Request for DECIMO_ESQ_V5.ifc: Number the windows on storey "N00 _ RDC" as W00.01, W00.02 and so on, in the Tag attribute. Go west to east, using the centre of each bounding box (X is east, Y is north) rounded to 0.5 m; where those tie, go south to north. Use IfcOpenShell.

First a look at what the model holds.

```python
import ifcopenshell
import ifcopenshell.util.element
import ifcopenshell.util.placement

model = ifcopenshell.open("DECIMO_ESQ_V5.ifc")
print(model.schema)
storey = next(s for s in model.by_type("IfcBuildingStorey") if s.Name == "N00 _ RDC")
windows = [e for e in ifcopenshell.util.element.get_decomposition(storey) if e.is_a("IfcWindow")]
for e in sorted(windows, key=lambda e: e.id()):
    origin = ifcopenshell.util.placement.get_local_placement(e.ObjectPlacement)[:3, 3]
    print(e.id(), e.Tag, e.Name, origin.round(2) + 0.0, sep=" | ")
```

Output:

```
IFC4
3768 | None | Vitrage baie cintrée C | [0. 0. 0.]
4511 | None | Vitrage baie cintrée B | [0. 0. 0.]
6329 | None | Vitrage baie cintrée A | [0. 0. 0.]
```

```python
import ifcopenshell
import ifcopenshell.geom
import ifcopenshell.util.element
import ifcopenshell.util.shape

model = ifcopenshell.open("DECIMO_ESQ_V5.ifc")
settings = ifcopenshell.geom.settings()
settings.set("use-world-coords", True)


def centre(element):
    shape = ifcopenshell.geom.create_shape(settings, element)
    return ifcopenshell.util.shape.get_bbox_centroid(shape.geometry)


storey = next(s for s in model.by_type("IfcBuildingStorey") if s.Name == "N00 _ RDC")
windows = [e for e in ifcopenshell.util.element.get_decomposition(storey) if e.is_a("IfcWindow")]

# Insertion points can sit at a corner or the storey origin, so sort by the geometry (in metres).
centres = {e: centre(e) for e in windows}
windows.sort(key=lambda e: (round(centres[e][0] / 0.5), centres[e][1]))

for i, e in enumerate(windows, start=1):
    number = f"W00.{i:02d}"
    e.Tag = number
    print(e.id(), number)

model.write("DECIMO_ESQ_V5_updated.ifc")
```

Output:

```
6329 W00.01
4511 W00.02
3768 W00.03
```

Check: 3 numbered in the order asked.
